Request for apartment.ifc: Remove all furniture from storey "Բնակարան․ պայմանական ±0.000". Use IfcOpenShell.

First a look at what the model holds.

```python
import ifcopenshell
import ifcopenshell.util.element

model = ifcopenshell.open("apartment.ifc")
print(model.schema)
storey = next(s for s in model.by_type("IfcBuildingStorey") if s.Name == "Բնակարան․ պայմանական ±0.000")
furniture = [e for e in ifcopenshell.util.element.get_decomposition(storey) if e.is_a("IfcFurnishingElement")]
seen = {}
for e in furniture:
    element_type = ifcopenshell.util.element.get_type(e)
    name = element_type.Name if element_type not in (None, e) else None
    seen[name] = seen.get(name, 0) + 1
for name, count in sorted(seen.items(), key=str):
    print(count, "x", name)
```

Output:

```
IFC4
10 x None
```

```python
import ifcopenshell
import ifcopenshell.api.root
import ifcopenshell.util.element

model = ifcopenshell.open("apartment.ifc")

storey = next(s for s in model.by_type("IfcBuildingStorey") if s.Name == "Բնակարան․ պայմանական ±0.000")
furniture = [e for e in ifcopenshell.util.element.get_decomposition(storey) if e.is_a("IfcFurnishingElement")]

for e in furniture:
    ifcopenshell.api.root.remove_product(model, product=e)
print(len(furniture), "removed")

model.write("apartment-out.ifc")
```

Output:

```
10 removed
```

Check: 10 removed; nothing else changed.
